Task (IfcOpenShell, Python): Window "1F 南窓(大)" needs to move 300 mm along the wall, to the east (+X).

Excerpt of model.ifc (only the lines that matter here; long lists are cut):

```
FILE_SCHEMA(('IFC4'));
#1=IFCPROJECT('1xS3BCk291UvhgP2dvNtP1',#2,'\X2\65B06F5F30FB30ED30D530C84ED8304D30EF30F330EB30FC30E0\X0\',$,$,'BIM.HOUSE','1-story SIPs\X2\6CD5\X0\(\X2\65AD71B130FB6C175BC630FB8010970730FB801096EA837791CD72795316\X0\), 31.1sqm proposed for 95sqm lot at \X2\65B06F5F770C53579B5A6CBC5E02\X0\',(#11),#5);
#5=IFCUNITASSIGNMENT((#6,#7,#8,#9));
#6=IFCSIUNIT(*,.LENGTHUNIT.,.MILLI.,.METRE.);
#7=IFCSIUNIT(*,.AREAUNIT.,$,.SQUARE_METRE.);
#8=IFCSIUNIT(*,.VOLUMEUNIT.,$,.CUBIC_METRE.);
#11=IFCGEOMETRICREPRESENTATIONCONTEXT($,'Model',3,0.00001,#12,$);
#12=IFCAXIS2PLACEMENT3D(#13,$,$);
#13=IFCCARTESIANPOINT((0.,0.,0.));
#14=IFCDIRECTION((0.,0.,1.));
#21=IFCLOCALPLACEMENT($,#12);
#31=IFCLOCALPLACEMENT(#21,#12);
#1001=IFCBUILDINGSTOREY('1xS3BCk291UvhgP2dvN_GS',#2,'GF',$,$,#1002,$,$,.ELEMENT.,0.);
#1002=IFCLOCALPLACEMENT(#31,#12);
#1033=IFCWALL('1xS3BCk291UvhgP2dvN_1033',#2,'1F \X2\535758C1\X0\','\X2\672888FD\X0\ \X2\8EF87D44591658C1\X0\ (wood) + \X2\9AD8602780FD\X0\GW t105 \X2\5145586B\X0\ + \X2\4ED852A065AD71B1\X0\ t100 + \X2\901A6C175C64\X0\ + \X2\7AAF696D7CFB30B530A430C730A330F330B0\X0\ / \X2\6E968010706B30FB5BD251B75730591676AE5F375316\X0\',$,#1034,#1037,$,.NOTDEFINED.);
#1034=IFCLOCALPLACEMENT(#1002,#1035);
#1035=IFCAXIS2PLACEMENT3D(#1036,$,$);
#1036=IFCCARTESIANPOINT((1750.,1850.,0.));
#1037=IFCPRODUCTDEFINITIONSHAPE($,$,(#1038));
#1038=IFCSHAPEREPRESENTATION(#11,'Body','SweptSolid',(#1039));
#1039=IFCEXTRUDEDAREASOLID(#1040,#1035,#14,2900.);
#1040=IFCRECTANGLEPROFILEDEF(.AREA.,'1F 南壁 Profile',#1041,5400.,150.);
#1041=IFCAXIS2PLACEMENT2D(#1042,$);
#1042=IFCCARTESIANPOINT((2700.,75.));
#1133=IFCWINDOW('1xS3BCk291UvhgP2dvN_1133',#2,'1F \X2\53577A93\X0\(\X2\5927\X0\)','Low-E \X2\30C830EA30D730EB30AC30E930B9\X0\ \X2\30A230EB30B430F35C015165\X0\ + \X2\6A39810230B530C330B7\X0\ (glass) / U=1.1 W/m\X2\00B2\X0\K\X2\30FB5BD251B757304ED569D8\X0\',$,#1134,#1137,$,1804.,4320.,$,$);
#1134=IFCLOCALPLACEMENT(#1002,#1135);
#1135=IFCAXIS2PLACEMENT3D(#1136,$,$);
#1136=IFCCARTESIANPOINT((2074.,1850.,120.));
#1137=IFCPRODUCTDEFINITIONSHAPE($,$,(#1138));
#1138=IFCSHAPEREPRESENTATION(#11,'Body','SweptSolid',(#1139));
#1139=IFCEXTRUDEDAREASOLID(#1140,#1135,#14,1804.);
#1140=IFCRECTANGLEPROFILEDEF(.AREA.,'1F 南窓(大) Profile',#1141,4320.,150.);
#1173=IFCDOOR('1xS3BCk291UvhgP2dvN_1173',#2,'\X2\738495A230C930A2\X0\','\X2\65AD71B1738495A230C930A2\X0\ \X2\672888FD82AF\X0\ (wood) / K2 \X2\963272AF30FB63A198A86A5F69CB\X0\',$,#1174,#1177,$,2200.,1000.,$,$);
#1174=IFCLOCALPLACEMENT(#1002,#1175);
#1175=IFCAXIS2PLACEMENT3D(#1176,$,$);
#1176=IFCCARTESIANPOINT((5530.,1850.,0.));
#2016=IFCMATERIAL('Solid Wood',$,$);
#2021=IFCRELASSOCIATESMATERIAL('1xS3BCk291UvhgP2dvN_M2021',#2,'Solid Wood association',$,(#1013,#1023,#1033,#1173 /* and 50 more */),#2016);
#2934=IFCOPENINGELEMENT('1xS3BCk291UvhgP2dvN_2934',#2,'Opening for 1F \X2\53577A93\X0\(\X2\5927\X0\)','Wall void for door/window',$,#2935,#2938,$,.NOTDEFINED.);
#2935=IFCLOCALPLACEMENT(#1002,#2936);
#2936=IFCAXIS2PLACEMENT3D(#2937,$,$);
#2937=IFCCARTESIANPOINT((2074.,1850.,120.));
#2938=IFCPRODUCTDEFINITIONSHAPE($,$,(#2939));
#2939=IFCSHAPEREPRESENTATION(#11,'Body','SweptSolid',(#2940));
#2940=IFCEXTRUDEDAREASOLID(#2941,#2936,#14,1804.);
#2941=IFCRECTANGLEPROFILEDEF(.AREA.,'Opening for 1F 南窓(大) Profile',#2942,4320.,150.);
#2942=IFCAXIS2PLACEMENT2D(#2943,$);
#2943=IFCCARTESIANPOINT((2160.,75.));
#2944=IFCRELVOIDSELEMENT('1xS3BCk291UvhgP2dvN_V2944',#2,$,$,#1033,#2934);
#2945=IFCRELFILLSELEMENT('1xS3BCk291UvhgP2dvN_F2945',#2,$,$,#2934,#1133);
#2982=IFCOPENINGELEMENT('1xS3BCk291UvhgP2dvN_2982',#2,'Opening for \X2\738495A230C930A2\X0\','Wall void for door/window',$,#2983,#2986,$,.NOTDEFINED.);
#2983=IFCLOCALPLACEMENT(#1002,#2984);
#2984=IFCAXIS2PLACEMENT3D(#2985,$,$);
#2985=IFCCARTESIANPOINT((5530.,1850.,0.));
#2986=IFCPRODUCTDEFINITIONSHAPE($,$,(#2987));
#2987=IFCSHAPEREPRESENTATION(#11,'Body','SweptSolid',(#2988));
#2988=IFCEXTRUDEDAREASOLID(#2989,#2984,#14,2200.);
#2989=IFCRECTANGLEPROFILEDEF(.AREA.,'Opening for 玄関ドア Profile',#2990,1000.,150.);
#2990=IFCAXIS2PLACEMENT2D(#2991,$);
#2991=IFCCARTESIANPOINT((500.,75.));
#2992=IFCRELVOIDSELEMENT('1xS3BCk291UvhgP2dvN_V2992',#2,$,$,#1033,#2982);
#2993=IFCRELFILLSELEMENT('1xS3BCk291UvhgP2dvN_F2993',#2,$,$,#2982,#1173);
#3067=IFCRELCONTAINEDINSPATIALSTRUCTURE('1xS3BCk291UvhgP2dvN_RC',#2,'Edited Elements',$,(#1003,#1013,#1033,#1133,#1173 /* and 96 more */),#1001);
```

```python
import ifcopenshell
import ifcopenshell.api.geometry
import ifcopenshell.util.placement

model = ifcopenshell.open("model.ifc")

window = model.by_id(1133)
opening = window.FillsVoids[0].RelatingOpeningElement
wall = opening.VoidsElements[0].RelatingBuildingElement

wall_matrix = ifcopenshell.util.placement.get_local_placement(wall.ObjectPlacement)
shift = wall_matrix[:3, 0] * 300.0
before = ifcopenshell.util.placement.get_local_placement(window.ObjectPlacement)[:3, 3].copy()

# The window is not placed relative to its opening, so move both.
for product in (opening, window):
    matrix = ifcopenshell.util.placement.get_local_placement(product.ObjectPlacement)
    matrix[:3, 3] += shift
    ifcopenshell.api.geometry.edit_object_placement(model, product=product, matrix=matrix, is_si=False)

after = ifcopenshell.util.placement.get_local_placement(window.ObjectPlacement)[:3, 3]
print("window moved by", (after - before).round(3) + 0.0)

model.write("model_v2.ifc")
```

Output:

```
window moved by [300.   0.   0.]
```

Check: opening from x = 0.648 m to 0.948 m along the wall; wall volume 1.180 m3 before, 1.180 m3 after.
